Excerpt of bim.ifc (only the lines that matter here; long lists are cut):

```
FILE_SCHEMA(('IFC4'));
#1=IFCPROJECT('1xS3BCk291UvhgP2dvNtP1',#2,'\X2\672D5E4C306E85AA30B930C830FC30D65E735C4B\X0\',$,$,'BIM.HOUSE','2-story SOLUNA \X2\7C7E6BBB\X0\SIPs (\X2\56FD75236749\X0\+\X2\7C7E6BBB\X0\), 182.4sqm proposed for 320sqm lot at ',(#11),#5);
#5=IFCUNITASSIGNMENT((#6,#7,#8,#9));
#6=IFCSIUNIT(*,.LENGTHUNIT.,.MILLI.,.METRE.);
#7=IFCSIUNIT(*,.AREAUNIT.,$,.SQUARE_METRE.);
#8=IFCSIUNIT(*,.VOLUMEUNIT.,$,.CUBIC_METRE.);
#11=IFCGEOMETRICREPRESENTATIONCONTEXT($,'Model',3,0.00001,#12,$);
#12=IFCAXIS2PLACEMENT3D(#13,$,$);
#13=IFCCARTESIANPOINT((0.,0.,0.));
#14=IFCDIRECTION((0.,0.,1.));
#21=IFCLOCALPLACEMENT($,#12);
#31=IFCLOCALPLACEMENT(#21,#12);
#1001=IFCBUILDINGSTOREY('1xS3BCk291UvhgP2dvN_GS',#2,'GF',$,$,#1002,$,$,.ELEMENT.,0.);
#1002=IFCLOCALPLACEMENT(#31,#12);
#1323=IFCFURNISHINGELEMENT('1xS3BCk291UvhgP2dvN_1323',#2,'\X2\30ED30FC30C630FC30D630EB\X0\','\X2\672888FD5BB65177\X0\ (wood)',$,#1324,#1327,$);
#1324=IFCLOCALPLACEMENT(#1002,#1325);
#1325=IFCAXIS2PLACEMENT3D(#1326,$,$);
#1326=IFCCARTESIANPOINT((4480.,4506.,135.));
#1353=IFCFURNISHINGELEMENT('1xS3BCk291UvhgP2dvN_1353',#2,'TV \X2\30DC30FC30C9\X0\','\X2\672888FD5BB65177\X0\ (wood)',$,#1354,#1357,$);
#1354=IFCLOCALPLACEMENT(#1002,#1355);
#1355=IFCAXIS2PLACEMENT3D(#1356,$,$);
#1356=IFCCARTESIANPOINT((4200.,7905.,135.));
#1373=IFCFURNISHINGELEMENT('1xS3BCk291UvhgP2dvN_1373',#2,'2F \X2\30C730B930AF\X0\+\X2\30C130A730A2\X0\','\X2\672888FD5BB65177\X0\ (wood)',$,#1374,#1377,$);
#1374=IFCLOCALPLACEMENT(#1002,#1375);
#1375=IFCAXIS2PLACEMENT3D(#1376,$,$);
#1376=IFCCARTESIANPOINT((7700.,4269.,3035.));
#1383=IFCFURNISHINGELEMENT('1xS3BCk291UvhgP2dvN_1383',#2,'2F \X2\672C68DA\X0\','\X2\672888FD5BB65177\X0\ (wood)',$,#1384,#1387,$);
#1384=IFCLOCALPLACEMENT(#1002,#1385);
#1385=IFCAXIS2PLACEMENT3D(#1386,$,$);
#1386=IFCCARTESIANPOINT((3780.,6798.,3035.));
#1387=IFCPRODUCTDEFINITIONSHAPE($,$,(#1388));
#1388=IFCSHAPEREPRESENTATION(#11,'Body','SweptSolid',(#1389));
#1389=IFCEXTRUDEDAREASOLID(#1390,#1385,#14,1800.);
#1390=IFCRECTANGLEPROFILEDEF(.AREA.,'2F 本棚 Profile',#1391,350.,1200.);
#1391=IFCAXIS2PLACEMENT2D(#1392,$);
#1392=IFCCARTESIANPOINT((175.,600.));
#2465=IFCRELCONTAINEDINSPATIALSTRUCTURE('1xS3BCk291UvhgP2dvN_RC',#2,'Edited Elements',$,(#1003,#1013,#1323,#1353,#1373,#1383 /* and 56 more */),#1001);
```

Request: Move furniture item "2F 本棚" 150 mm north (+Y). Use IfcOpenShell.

```python
import ifcopenshell
import ifcopenshell.api.geometry
import ifcopenshell.util.placement

model = ifcopenshell.open("bim.ifc")

item = model.by_guid("1xS3BCk291UvhgP2dvN_1383")
matrix = ifcopenshell.util.placement.get_local_placement(item.ObjectPlacement)
matrix[1, 3] += 150.0
ifcopenshell.api.geometry.edit_object_placement(model, product=item, matrix=matrix, is_si=False)

print(ifcopenshell.util.placement.get_local_placement(item.ObjectPlacement).round(3) + 0.0)

model.write("bim_edited.ifc")
```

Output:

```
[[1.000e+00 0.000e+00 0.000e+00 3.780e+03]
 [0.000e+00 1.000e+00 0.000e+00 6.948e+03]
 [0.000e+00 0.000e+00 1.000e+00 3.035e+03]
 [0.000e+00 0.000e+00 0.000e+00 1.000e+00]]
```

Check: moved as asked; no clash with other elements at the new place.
